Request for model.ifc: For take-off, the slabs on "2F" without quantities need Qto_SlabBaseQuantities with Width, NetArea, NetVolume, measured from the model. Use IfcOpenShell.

First a look at what the model holds.

```python
import ifcopenshell
import ifcopenshell.util.element
import ifcopenshell.util.unit

model = ifcopenshell.open("model.ifc")
print(model.schema)
for unit_type in ("LENGTHUNIT", "AREAUNIT", "VOLUMEUNIT"):
    print(unit_type, ifcopenshell.util.unit.calculate_unit_scale(model, unit_type))
storey = next(s for s in model.by_type("IfcBuildingStorey") if s.Name == "2F")
slabs = [e for e in ifcopenshell.util.element.get_decomposition(storey) if e.is_a("IfcSlab")]
for e in sorted(slabs, key=lambda e: e.id()):
    print(e.id(), e.is_a(), e.Name, list(ifcopenshell.util.element.get_psets(e, qtos_only=True)), sep=" | ")
```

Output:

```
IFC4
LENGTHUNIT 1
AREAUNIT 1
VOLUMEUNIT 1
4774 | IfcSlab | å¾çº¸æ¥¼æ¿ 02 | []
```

```python
import ifcopenshell
import ifcopenshell.api.pset
import ifcopenshell.geom
import ifcopenshell.util.element
import ifcopenshell.util.shape
import ifcopenshell.util.unit

model = ifcopenshell.open("model.ifc")
unit_scale = ifcopenshell.util.unit.calculate_unit_scale(model)
area_scale = ifcopenshell.util.unit.calculate_unit_scale(model, "AREAUNIT")
volume_scale = ifcopenshell.util.unit.calculate_unit_scale(model, "VOLUMEUNIT")
settings = ifcopenshell.geom.settings()

storey = next(s for s in model.by_type("IfcBuildingStorey") if s.Name == "2F")
slabs = [e for e in ifcopenshell.util.element.get_decomposition(storey) if e.is_a("IfcSlab")]

for e in sorted(slabs, key=lambda e: e.id()):
    if ifcopenshell.util.element.get_psets(e, qtos_only=True, should_inherit=False):
        continue
    # Geometry comes back in metres, in the element's own axes.
    shape = ifcopenshell.geom.create_shape(settings, e)
    values = {
        "Width": ifcopenshell.util.shape.get_z(shape.geometry) / unit_scale,
        "NetArea": ifcopenshell.util.shape.get_footprint_area(shape.geometry) / area_scale,
        "NetVolume": ifcopenshell.util.shape.get_volume(shape.geometry) / volume_scale,
    }
    qto = ifcopenshell.api.pset.add_qto(model, product=e, name="Qto_SlabBaseQuantities")
    ifcopenshell.api.pset.edit_qto(model, qto=qto, properties=values)
    print(e.id(), {k: round(v, 3) for k, v in values.items()})

model.write("model_rev.ifc")
```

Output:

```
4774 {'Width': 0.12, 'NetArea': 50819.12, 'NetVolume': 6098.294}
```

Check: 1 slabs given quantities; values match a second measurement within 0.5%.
